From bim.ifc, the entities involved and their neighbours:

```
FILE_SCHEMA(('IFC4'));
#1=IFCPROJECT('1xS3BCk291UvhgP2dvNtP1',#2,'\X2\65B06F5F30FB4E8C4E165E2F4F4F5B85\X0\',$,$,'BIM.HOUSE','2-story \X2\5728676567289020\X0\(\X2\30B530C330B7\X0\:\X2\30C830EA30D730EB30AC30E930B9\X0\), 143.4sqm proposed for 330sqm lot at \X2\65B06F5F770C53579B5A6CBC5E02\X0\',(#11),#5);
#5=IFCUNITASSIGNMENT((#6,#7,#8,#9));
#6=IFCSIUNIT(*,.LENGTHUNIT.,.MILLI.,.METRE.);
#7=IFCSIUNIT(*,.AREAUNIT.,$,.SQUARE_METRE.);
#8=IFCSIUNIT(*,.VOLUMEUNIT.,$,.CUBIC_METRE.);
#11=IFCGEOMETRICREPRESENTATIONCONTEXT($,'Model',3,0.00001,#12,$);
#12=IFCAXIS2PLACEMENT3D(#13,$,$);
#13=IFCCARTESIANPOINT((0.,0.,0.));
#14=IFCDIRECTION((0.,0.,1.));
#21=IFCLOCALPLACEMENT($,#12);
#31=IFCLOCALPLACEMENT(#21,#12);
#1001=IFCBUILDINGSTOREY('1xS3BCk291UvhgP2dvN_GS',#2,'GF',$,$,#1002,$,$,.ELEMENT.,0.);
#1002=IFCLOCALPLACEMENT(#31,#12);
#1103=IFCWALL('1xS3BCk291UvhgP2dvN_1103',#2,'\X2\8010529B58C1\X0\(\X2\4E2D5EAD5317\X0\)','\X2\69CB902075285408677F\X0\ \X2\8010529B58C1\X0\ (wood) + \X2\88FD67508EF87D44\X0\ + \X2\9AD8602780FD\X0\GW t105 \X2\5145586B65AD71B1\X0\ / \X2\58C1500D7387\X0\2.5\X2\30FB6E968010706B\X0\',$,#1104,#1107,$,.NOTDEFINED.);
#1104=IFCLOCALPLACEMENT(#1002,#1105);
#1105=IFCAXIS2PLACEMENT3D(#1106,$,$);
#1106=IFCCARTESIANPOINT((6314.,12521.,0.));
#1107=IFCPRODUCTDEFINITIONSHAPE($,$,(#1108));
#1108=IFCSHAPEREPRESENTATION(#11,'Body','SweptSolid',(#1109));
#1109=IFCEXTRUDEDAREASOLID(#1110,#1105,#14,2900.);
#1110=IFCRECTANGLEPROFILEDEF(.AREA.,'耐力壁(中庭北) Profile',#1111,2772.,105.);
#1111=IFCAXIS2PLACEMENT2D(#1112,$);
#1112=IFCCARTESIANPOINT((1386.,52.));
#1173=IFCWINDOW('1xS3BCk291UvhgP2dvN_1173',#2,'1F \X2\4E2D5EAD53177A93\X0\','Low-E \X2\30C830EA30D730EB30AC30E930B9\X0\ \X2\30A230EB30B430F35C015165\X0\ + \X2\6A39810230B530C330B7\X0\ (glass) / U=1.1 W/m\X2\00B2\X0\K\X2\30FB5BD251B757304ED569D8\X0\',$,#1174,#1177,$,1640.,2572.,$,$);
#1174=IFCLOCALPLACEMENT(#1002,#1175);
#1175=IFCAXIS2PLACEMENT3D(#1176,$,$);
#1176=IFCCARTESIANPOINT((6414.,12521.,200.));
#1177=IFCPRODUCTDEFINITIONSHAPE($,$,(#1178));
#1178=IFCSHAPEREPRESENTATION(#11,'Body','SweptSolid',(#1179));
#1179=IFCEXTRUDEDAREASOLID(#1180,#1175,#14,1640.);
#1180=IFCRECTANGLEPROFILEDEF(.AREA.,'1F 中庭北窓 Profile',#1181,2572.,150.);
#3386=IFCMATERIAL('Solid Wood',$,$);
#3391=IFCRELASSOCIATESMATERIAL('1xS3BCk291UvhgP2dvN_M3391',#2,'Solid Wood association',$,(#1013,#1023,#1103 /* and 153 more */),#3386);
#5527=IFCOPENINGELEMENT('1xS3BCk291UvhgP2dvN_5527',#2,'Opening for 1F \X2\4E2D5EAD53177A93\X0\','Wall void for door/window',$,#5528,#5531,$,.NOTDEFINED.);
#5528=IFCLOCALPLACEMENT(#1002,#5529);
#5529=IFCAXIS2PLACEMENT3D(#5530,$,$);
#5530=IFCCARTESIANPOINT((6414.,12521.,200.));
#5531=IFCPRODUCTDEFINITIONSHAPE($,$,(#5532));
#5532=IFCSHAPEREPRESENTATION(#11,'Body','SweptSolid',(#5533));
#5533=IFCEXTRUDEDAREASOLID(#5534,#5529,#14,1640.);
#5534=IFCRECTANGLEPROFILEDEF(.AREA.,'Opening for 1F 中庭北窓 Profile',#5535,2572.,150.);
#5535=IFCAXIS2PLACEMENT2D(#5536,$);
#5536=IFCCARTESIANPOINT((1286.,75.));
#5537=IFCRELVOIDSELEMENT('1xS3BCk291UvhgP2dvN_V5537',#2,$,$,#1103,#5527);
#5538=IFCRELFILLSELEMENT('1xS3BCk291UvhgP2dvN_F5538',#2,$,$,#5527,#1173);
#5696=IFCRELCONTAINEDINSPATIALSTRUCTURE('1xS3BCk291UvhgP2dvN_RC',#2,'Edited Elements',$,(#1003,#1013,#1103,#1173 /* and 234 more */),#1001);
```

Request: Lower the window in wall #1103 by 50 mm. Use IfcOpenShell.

```python
import numpy as np
import ifcopenshell
import ifcopenshell.api.geometry
import ifcopenshell.util.placement
import ifcopenshell.util.unit

model = ifcopenshell.open("bim.ifc")
unit_scale = ifcopenshell.util.unit.calculate_unit_scale(model)

window = model.by_guid("1xS3BCk291UvhgP2dvN_1173")
opening = window.FillsVoids[0].RelatingOpeningElement
dz = -50.0

shift = np.array([0.0, 0.0, dz])
# The window is not placed relative to its opening, so move both.
for product in (opening, window):
    matrix = ifcopenshell.util.placement.get_local_placement(product.ObjectPlacement)
    matrix[:3, 3] += shift
    ifcopenshell.api.geometry.edit_object_placement(model, product=product, matrix=matrix, is_si=False)

print(f"moved by {dz * unit_scale:+.3f} m")

model.write("bim_edited.ifc")
```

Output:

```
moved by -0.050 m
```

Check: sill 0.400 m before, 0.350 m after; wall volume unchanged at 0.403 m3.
